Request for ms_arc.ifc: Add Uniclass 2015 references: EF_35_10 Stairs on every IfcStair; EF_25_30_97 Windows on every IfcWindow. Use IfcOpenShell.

First a look at what the model holds.

```python
import ifcopenshell

model = ifcopenshell.open("ms_arc.ifc")
print(model.schema)
print("classifications:", [c.Name for c in model.by_type("IfcClassification")])
for ifc_class in ("IfcDoor", "IfcRoof", "IfcStair", "IfcWall", "IfcWindow"):
    print(ifc_class, len(model.by_type(ifc_class)))
```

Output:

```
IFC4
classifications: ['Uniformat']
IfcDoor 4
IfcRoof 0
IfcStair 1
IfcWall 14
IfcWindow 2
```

```python
import ifcopenshell
import ifcopenshell.api.classification

model = ifcopenshell.open("ms_arc.ifc")

system = ifcopenshell.api.classification.add_classification(model, classification="Uniclass 2015")

codes = {
    "IfcStair": ("EF_35_10", "Stairs"),
    "IfcWindow": ("EF_25_30_97", "Windows"),
}
for ifc_class, (code, name) in codes.items():
    products = model.by_type(ifc_class)
    ifcopenshell.api.classification.add_reference(
        model, products=products, classification=system, identification=code, name=name
    )
    print(code, len(products))

model.write("ms_arc_edited.ifc")
```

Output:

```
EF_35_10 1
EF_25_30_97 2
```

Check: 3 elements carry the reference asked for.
